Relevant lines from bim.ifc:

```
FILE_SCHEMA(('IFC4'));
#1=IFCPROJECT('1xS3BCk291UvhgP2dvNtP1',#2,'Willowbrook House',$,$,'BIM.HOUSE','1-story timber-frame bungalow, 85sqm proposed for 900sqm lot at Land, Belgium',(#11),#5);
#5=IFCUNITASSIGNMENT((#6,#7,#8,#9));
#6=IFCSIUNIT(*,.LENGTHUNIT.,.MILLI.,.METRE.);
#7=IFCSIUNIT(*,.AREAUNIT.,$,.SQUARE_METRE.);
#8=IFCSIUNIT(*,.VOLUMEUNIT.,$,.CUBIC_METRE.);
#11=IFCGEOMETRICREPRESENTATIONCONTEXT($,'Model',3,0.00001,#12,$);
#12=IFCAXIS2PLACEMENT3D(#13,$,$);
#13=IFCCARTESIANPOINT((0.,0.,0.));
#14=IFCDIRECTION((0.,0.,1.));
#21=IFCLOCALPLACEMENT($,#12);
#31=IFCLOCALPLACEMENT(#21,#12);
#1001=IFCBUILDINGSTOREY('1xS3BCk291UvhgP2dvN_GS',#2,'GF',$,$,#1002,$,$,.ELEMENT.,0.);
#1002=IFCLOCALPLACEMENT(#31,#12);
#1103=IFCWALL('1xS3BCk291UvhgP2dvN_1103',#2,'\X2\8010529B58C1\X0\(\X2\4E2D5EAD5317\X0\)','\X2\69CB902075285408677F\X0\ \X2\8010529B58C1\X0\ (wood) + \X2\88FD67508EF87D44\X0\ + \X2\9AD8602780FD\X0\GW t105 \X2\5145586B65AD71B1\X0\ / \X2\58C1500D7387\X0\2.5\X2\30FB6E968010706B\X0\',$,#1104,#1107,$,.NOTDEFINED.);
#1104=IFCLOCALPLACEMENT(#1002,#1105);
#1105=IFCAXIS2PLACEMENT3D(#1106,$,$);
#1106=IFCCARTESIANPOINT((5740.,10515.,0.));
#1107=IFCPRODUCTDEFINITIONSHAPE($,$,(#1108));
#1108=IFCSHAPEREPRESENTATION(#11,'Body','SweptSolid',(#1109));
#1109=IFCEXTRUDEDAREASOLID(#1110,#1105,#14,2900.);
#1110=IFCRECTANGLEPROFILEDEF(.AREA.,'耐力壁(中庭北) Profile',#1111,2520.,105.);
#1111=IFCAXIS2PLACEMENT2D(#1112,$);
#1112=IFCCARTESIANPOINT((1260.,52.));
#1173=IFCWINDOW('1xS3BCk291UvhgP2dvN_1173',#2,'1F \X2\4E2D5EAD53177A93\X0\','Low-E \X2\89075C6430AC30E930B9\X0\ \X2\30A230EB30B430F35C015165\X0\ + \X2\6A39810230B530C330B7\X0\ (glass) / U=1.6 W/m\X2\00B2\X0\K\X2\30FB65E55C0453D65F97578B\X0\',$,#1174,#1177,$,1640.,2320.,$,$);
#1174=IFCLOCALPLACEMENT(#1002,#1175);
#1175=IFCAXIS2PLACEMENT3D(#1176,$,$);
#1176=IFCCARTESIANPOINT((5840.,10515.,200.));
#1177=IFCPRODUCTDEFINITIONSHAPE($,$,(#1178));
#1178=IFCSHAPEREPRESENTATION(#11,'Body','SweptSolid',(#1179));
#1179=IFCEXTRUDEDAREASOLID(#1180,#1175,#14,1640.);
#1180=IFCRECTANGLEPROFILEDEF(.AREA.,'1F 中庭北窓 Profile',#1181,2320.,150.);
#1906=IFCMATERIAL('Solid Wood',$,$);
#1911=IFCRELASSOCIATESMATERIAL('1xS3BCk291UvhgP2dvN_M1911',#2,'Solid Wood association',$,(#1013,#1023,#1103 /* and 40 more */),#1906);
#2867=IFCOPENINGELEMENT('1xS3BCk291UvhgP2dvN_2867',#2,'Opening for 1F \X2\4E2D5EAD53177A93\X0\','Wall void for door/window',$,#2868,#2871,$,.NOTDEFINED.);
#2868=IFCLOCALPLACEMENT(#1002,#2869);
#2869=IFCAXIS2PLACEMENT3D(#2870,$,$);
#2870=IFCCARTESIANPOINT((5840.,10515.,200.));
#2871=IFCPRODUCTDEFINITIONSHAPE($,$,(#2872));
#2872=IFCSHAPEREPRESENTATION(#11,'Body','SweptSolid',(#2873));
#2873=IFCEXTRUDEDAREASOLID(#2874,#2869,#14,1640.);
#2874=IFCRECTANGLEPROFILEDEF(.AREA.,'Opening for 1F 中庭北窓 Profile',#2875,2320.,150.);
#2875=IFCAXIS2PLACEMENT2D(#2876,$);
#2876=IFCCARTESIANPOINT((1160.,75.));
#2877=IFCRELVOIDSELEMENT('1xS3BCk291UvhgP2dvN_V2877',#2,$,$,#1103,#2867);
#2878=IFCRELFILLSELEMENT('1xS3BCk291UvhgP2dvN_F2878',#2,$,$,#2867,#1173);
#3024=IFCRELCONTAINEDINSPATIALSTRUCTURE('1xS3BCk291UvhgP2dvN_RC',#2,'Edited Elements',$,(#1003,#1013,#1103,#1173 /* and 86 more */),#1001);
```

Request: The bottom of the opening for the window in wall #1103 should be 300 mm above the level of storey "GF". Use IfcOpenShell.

```python
import numpy as np
import ifcopenshell
import ifcopenshell.api.geometry
import ifcopenshell.geom
import ifcopenshell.util.element
import ifcopenshell.util.placement
import ifcopenshell.util.shape
import ifcopenshell.util.unit

model = ifcopenshell.open("bim.ifc")
unit_scale = ifcopenshell.util.unit.calculate_unit_scale(model)

window = model.by_guid("1xS3BCk291UvhgP2dvN_1173")
opening = window.FillsVoids[0].RelatingOpeningElement
storey = ifcopenshell.util.element.get_container(window, ifc_class="IfcBuildingStorey")
level = ifcopenshell.util.placement.get_local_placement(storey.ObjectPlacement)[2, 3]

# The opening's origin need not be at the sill, so measure its lowest point.
shape = ifcopenshell.geom.create_shape(ifcopenshell.geom.settings(), opening)
bottom = ifcopenshell.util.shape.get_shape_bottom_elevation(shape, shape.geometry) / unit_scale
dz = level + 0.3 / unit_scale - bottom

shift = np.array([0.0, 0.0, dz])
# The window is not placed relative to its opening, so move both.
for product in (opening, window):
    matrix = ifcopenshell.util.placement.get_local_placement(product.ObjectPlacement)
    matrix[:3, 3] += shift
    ifcopenshell.api.geometry.edit_object_placement(model, product=product, matrix=matrix, is_si=False)

print(f"moved by {dz * unit_scale:+.3f} m")

model.write("bim-out.ifc")
```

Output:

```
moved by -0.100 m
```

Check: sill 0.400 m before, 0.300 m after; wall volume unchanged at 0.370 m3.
